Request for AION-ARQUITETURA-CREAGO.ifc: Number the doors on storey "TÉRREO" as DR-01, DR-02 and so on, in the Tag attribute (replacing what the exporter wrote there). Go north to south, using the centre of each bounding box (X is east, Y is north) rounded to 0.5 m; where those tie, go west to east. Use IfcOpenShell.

First a look at what the model holds.

```python
import ifcopenshell
import ifcopenshell.util.element
import ifcopenshell.util.placement

model = ifcopenshell.open("AION-ARQUITETURA-CREAGO.ifc")
print(model.schema)
storey = next(s for s in model.by_type("IfcBuildingStorey") if s.Name == "TÉRREO")
doors = [e for e in ifcopenshell.util.element.get_decomposition(storey) if e.is_a("IfcDoor")]
for e in sorted(doors, key=lambda e: e.id()):
    origin = ifcopenshell.util.placement.get_local_placement(e.ObjectPlacement)[:3, 3]
    print(e.id(), e.Tag, e.Name, origin.round(2) + 0.0, sep=" | ")
```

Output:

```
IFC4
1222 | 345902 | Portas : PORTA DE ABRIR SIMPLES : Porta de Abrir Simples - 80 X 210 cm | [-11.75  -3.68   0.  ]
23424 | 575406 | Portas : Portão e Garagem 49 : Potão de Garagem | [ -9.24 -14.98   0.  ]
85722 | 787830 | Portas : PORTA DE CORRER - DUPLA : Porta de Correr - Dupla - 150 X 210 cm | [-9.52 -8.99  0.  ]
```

```python
import ifcopenshell
import ifcopenshell.geom
import ifcopenshell.util.element
import ifcopenshell.util.shape

model = ifcopenshell.open("AION-ARQUITETURA-CREAGO.ifc")
settings = ifcopenshell.geom.settings()
settings.set("use-world-coords", True)


def centre(element):
    shape = ifcopenshell.geom.create_shape(settings, element)
    return ifcopenshell.util.shape.get_bbox_centroid(shape.geometry)


storey = next(s for s in model.by_type("IfcBuildingStorey") if s.Name == "TÉRREO")
doors = [e for e in ifcopenshell.util.element.get_decomposition(storey) if e.is_a("IfcDoor")]

# Insertion points can sit at a corner or the storey origin, so sort by the geometry (in metres).
centres = {e: centre(e) for e in doors}
doors.sort(key=lambda e: (-round(centres[e][1] / 0.5), centres[e][0]))

for i, e in enumerate(doors, start=1):
    number = f"DR-{i:02d}"
    e.Tag = number
    print(e.id(), number)

model.write("AION-ARQUITETURA-CREAGO_updated.ifc")
```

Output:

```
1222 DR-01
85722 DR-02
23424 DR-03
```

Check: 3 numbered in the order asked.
